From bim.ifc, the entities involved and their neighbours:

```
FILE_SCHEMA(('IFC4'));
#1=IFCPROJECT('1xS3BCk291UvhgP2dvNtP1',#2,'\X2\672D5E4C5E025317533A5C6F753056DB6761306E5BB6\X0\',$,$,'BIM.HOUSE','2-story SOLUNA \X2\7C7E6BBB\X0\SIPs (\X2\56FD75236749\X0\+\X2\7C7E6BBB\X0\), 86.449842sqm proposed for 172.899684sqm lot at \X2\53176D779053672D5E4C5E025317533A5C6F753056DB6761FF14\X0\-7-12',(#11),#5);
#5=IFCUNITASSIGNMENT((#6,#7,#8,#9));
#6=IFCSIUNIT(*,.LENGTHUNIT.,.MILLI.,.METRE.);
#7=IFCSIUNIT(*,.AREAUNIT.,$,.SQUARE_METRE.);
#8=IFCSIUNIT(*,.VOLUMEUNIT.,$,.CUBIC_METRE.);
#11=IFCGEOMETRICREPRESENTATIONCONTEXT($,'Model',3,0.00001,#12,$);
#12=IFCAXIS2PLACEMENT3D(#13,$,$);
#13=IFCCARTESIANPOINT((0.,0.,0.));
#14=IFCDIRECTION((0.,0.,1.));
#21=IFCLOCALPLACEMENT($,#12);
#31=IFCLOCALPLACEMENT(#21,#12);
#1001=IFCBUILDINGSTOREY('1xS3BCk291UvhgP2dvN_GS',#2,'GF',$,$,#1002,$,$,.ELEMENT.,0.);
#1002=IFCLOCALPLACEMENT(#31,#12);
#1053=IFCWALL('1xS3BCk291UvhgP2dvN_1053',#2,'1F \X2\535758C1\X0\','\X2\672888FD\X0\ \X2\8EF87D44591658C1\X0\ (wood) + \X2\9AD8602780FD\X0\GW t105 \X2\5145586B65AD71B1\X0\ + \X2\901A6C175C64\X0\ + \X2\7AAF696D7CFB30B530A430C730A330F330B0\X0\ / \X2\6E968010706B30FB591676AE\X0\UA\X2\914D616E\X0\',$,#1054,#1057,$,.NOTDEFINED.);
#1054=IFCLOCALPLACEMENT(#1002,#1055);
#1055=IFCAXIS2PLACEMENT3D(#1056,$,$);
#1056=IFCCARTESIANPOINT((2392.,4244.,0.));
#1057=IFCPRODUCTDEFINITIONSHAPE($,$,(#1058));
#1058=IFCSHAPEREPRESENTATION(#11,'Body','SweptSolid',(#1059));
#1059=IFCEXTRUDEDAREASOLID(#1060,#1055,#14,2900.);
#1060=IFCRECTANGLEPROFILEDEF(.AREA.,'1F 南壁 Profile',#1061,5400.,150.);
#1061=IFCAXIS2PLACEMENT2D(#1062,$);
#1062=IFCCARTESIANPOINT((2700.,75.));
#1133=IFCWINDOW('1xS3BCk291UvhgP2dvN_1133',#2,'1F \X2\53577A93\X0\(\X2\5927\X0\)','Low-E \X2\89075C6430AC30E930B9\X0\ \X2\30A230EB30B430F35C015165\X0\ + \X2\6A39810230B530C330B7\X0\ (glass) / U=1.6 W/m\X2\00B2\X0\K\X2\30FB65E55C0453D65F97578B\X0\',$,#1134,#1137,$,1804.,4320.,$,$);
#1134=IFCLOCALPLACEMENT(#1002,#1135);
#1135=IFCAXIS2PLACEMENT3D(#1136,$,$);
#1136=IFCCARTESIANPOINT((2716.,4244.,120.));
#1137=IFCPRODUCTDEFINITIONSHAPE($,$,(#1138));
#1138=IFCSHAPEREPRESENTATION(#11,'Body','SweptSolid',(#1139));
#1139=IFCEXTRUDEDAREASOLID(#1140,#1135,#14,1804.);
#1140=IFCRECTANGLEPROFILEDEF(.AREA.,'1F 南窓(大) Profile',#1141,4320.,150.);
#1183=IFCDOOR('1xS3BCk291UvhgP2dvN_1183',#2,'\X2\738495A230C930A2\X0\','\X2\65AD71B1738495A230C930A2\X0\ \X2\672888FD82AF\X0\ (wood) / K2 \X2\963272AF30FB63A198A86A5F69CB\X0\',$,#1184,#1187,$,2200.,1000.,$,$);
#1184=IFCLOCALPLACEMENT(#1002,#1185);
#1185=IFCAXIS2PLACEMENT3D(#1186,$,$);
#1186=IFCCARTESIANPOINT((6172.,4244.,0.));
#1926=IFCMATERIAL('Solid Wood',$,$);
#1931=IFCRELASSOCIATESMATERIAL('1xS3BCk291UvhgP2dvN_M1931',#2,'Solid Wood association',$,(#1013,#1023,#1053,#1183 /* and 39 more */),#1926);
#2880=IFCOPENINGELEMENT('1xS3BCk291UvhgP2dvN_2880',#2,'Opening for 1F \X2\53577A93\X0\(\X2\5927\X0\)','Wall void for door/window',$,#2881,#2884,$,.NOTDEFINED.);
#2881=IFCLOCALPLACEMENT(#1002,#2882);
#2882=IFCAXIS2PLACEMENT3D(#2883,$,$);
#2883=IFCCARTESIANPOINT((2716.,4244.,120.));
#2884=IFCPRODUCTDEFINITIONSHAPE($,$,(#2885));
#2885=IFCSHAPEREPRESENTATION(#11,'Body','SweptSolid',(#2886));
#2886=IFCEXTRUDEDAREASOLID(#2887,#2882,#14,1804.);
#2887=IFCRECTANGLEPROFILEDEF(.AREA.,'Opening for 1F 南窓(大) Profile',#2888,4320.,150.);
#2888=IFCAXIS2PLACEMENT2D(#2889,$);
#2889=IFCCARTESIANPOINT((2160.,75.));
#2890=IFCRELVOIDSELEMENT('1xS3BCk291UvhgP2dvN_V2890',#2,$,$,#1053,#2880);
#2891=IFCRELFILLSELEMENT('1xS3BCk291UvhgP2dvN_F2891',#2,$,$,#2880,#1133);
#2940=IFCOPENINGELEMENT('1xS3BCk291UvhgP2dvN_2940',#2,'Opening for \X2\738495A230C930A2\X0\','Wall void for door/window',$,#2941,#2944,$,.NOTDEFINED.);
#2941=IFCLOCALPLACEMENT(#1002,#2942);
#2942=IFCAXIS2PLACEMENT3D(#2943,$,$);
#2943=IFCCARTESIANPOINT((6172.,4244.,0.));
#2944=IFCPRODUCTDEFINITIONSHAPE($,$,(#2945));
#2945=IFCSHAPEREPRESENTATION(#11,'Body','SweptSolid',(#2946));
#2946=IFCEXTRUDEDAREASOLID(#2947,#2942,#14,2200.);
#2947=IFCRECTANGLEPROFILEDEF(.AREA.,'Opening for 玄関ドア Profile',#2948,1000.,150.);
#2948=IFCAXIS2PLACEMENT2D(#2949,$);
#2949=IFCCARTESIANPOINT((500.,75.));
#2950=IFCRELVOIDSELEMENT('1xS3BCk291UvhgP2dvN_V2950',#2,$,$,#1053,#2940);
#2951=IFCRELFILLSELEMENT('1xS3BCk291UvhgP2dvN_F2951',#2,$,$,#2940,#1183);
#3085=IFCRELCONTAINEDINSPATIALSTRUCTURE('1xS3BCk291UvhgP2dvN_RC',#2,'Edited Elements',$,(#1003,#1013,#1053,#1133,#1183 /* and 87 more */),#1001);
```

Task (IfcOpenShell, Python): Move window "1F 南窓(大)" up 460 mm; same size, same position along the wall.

```python
import numpy as np
import ifcopenshell
import ifcopenshell.api.geometry
import ifcopenshell.util.placement
import ifcopenshell.util.unit

model = ifcopenshell.open("bim.ifc")
unit_scale = ifcopenshell.util.unit.calculate_unit_scale(model)

window = model.by_guid("1xS3BCk291UvhgP2dvN_1133")
opening = window.FillsVoids[0].RelatingOpeningElement
dz = 0.46 / unit_scale

shift = np.array([0.0, 0.0, dz])
# The window is not placed relative to its opening, so move both.
for product in (opening, window):
    matrix = ifcopenshell.util.placement.get_local_placement(product.ObjectPlacement)
    matrix[:3, 3] += shift
    ifcopenshell.api.geometry.edit_object_placement(model, product=product, matrix=matrix, is_si=False)

print(f"moved by {dz * unit_scale:+.3f} m")

model.write("bim-out.ifc")
```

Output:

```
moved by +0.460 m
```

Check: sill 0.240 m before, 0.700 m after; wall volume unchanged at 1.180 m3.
